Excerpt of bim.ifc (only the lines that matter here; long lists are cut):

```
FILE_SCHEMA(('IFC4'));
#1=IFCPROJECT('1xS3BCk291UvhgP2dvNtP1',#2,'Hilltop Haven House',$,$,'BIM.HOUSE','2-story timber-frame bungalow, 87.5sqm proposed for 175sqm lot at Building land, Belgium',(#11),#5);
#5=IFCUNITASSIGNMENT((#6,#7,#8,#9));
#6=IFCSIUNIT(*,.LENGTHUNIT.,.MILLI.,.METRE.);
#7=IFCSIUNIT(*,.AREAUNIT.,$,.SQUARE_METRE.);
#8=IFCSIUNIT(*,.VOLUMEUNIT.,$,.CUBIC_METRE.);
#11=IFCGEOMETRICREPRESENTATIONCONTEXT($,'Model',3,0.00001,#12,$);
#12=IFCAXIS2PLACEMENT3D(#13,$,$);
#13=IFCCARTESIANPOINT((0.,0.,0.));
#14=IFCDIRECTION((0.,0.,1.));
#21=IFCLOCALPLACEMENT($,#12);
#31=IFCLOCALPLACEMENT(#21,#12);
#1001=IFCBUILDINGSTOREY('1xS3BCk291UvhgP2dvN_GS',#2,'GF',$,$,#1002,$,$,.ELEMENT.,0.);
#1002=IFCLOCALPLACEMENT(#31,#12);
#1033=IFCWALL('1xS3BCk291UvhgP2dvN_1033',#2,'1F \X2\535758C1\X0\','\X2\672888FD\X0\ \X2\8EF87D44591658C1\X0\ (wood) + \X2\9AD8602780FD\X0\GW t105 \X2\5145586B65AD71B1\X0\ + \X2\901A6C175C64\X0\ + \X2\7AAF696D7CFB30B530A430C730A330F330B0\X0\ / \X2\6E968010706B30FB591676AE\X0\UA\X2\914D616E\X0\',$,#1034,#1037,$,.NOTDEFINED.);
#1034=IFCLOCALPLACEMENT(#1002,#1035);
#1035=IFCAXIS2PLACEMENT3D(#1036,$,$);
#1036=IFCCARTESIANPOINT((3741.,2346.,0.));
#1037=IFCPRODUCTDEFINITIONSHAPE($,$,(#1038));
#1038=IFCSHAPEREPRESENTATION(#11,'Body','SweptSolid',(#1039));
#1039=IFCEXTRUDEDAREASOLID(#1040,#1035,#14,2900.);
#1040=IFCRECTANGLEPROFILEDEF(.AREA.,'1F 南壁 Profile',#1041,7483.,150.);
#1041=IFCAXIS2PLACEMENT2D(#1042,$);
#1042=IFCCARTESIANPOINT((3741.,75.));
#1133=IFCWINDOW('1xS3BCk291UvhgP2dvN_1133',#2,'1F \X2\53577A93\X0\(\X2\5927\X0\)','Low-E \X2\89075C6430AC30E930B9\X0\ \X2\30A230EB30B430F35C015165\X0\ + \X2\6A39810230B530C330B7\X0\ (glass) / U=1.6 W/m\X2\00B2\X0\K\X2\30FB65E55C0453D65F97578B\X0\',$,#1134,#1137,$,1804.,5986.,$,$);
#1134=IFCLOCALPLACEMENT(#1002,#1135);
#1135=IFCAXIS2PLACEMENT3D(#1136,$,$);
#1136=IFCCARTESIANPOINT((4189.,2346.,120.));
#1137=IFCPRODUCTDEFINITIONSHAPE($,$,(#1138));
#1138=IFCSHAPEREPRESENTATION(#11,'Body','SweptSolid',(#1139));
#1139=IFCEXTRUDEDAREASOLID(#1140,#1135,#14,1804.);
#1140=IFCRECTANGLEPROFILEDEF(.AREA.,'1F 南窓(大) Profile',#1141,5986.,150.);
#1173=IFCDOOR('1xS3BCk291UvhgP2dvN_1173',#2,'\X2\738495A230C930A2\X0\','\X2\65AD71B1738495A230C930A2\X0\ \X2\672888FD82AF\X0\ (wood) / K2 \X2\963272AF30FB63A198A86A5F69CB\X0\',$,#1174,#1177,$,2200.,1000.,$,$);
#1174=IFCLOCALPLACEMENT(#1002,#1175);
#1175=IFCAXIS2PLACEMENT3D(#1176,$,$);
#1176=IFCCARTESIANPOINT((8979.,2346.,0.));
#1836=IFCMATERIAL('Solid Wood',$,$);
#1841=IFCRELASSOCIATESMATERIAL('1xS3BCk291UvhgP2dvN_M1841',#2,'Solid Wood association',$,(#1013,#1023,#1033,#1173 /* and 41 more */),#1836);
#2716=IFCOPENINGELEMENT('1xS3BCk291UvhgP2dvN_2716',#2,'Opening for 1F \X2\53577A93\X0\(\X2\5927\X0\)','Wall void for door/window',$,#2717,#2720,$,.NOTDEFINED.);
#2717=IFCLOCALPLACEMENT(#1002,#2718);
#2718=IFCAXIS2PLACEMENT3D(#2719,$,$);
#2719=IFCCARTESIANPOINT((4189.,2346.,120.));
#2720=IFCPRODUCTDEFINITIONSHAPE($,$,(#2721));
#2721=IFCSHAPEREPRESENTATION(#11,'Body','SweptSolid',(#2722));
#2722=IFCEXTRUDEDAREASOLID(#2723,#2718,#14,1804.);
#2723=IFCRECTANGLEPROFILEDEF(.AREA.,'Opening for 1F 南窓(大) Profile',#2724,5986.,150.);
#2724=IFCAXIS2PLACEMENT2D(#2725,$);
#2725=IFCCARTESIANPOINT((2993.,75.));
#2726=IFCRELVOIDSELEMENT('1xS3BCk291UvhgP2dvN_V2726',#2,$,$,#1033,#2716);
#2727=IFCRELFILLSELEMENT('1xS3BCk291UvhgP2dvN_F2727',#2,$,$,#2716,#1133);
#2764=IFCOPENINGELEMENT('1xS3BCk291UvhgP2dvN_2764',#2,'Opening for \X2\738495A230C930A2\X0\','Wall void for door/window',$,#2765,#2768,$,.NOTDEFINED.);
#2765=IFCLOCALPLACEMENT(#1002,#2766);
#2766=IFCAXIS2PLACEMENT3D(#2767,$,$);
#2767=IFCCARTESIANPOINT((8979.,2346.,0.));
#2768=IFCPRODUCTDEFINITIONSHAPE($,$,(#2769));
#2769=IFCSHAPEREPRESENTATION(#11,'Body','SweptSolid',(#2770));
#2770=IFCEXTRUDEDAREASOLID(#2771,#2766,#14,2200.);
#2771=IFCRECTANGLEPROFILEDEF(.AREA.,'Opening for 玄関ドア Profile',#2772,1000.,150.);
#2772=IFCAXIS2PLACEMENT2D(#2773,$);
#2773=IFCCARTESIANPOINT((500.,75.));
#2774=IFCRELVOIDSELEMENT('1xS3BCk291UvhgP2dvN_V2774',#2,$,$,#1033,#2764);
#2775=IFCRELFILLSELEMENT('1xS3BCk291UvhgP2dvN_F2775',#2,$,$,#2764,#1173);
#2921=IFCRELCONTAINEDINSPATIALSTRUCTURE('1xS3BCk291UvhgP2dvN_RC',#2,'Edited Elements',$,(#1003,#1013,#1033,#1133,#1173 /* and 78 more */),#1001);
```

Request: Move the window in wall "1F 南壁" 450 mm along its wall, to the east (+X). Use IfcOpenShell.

```python
import ifcopenshell
import ifcopenshell.api.geometry
import ifcopenshell.util.placement
import ifcopenshell.util.unit

model = ifcopenshell.open("bim.ifc")
unit_scale = ifcopenshell.util.unit.calculate_unit_scale(model)

window = model.by_guid("1xS3BCk291UvhgP2dvN_1133")
opening = window.FillsVoids[0].RelatingOpeningElement
wall = opening.VoidsElements[0].RelatingBuildingElement

wall_matrix = ifcopenshell.util.placement.get_local_placement(wall.ObjectPlacement)
shift = wall_matrix[:3, 0] * 0.45 / unit_scale
before = ifcopenshell.util.placement.get_local_placement(window.ObjectPlacement)[:3, 3].copy()

# The window is not placed relative to its opening, so move both.
for product in (opening, window):
    matrix = ifcopenshell.util.placement.get_local_placement(product.ObjectPlacement)
    matrix[:3, 3] += shift
    ifcopenshell.api.geometry.edit_object_placement(model, product=product, matrix=matrix, is_si=False)

after = ifcopenshell.util.placement.get_local_placement(window.ObjectPlacement)[:3, 3]
print("window moved by", (after - before).round(3) + 0.0)

model.write("bim_updated.ifc")
```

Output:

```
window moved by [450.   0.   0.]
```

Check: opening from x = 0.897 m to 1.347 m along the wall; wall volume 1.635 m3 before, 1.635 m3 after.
